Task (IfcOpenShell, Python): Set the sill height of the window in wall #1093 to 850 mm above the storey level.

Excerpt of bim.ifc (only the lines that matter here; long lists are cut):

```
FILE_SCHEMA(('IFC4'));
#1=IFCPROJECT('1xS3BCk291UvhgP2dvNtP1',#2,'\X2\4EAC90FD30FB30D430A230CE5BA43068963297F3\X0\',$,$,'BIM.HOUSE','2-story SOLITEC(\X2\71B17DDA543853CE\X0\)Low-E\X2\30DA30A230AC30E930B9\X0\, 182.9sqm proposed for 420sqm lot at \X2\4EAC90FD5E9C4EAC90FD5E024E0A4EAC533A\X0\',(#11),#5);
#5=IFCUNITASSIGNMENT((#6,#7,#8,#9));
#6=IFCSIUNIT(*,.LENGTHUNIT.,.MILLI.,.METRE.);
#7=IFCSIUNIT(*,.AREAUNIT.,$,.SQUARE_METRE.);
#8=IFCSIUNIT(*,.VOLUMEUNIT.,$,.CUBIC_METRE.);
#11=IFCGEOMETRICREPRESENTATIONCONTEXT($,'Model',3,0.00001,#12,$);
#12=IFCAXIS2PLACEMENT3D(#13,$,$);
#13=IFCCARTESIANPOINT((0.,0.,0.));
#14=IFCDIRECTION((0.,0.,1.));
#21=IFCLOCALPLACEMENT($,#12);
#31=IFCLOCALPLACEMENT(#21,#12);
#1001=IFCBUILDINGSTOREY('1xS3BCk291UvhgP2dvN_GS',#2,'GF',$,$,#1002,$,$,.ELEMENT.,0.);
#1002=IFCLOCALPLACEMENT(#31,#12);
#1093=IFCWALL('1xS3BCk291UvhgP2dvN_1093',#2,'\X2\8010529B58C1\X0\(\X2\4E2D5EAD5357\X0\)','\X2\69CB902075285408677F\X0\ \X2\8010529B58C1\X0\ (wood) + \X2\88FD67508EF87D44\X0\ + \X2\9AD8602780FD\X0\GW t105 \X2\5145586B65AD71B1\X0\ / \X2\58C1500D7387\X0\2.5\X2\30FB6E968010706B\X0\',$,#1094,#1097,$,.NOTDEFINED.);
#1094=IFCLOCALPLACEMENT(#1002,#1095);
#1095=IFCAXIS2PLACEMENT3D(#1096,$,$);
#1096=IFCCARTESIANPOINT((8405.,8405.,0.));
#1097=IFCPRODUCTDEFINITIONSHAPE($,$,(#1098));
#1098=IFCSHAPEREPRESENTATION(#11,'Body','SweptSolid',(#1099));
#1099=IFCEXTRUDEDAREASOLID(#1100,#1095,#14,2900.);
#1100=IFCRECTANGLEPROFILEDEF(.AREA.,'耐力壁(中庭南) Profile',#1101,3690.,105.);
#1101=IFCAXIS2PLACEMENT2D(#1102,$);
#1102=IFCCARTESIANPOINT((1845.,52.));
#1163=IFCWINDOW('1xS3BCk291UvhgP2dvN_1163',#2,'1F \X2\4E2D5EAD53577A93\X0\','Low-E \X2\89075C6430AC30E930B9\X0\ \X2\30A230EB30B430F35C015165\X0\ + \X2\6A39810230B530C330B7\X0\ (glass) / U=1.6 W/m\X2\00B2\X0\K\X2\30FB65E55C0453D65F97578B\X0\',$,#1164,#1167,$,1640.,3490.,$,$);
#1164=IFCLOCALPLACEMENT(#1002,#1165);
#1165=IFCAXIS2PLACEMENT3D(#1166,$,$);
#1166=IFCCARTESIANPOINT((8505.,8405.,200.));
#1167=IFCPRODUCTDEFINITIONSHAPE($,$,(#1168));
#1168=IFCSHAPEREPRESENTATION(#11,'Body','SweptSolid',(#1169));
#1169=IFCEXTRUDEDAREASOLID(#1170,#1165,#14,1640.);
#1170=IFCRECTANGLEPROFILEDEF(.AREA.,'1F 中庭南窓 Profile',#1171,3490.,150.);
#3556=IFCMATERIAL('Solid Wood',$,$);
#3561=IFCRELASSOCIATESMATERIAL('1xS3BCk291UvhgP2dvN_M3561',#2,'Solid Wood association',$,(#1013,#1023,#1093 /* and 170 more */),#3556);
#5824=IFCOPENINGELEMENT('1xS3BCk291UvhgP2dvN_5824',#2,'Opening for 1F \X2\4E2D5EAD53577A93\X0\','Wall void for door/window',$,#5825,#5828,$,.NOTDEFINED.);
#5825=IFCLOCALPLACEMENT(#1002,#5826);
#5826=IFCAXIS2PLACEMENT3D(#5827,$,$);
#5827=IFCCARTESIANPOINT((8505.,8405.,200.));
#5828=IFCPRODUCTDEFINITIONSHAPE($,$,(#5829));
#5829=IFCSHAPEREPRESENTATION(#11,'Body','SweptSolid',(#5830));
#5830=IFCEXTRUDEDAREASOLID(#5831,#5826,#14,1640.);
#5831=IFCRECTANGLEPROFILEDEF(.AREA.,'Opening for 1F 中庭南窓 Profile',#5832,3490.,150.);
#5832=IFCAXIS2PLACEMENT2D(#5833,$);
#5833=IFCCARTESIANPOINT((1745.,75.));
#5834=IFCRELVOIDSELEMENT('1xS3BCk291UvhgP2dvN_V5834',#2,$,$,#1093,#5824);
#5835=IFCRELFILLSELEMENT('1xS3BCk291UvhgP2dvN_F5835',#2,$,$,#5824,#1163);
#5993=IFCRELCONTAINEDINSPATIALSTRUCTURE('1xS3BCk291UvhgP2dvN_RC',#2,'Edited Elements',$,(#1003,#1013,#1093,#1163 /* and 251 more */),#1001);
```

```python
import numpy as np
import ifcopenshell
import ifcopenshell.api.geometry
import ifcopenshell.geom
import ifcopenshell.util.element
import ifcopenshell.util.placement
import ifcopenshell.util.shape
import ifcopenshell.util.unit

model = ifcopenshell.open("bim.ifc")
unit_scale = ifcopenshell.util.unit.calculate_unit_scale(model)

window = model.by_guid("1xS3BCk291UvhgP2dvN_1163")
opening = window.FillsVoids[0].RelatingOpeningElement
storey = ifcopenshell.util.element.get_container(window, ifc_class="IfcBuildingStorey")
level = ifcopenshell.util.placement.get_local_placement(storey.ObjectPlacement)[2, 3]

# The opening's origin need not be at the sill, so measure its lowest point.
shape = ifcopenshell.geom.create_shape(ifcopenshell.geom.settings(), opening)
bottom = ifcopenshell.util.shape.get_shape_bottom_elevation(shape, shape.geometry) / unit_scale
dz = level + 850.0 - bottom

shift = np.array([0.0, 0.0, dz])
# The window is not placed relative to its opening, so move both.
for product in (opening, window):
    matrix = ifcopenshell.util.placement.get_local_placement(product.ObjectPlacement)
    matrix[:3, 3] += shift
    ifcopenshell.api.geometry.edit_object_placement(model, product=product, matrix=matrix, is_si=False)

print(f"moved by {dz * unit_scale:+.3f} m")

model.write("bim_edited.ifc")
```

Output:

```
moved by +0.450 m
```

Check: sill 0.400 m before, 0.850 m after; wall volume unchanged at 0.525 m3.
